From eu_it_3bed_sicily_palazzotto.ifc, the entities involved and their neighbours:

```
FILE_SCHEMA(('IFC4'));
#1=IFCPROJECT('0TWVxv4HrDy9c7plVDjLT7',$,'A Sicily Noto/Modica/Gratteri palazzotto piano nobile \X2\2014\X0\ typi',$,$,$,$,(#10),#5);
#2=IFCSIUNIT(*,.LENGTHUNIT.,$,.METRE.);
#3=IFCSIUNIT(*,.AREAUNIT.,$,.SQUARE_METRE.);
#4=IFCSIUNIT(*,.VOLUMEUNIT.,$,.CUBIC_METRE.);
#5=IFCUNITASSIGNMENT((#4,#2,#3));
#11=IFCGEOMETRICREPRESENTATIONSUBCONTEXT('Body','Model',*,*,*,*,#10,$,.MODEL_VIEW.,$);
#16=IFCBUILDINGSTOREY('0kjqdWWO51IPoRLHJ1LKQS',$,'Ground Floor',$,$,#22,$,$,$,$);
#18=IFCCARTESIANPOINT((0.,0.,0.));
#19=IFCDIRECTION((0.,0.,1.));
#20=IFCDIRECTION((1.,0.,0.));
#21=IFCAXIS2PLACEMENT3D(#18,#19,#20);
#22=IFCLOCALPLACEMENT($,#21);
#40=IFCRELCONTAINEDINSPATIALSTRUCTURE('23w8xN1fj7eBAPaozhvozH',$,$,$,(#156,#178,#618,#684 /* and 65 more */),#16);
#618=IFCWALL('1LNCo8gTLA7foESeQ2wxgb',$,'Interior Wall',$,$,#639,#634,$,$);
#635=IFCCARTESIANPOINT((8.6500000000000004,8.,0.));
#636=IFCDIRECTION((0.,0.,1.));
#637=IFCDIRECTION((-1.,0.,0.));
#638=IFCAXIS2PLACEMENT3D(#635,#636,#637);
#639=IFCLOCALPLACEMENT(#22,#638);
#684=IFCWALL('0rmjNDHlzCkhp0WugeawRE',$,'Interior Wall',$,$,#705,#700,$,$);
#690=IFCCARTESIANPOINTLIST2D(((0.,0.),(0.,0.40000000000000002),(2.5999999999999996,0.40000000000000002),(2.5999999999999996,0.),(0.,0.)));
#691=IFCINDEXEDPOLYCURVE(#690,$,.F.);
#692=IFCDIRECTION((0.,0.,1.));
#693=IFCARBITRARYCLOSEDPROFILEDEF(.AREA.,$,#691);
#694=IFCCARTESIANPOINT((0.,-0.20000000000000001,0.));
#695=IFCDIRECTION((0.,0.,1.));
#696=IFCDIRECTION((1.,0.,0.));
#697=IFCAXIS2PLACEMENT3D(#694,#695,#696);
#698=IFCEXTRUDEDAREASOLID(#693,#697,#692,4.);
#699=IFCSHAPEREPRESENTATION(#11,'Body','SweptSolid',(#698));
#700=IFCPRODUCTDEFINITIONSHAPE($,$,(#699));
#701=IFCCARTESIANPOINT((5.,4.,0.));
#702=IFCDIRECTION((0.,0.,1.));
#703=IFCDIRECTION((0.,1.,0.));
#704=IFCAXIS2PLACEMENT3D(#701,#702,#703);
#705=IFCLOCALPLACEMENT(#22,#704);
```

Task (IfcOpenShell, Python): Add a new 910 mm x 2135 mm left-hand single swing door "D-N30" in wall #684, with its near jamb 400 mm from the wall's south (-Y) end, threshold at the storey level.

```python
import numpy as np
import ifcopenshell
import ifcopenshell.api.feature
import ifcopenshell.api.geometry
import ifcopenshell.api.root
import ifcopenshell.api.spatial
import ifcopenshell.geom
import ifcopenshell.util.element
import ifcopenshell.util.placement
import ifcopenshell.util.representation
import ifcopenshell.util.shape
import ifcopenshell.util.unit

model = ifcopenshell.open("eu_it_3bed_sicily_palazzotto.ifc")
unit_scale = ifcopenshell.util.unit.calculate_unit_scale(model)
settings = ifcopenshell.geom.settings()


def volume(element):
    """Net volume in cubic metres, openings subtracted."""
    shape = ifcopenshell.geom.create_shape(settings, element)
    return ifcopenshell.util.shape.get_volume(shape.geometry)


wall = model.by_guid("0rmjNDHlzCkhp0WugeawRE")
storey = ifcopenshell.util.element.get_container(wall, ifc_class="IfcBuildingStorey")
context = ifcopenshell.util.representation.get_context(model, "Model", "Body", "MODEL_VIEW")
before = volume(wall)

width, height, from_end, sill = 0.91, 2.135, 0.4, 0.0  # metres

# The wall runs along its own X axis, and the end named is its -X end.
wall_shape = ifcopenshell.geom.create_shape(settings, wall)
x, y, z = ifcopenshell.util.shape.get_vertices(wall_shape.geometry).T
start = x.min() + from_end
face, thickness = float(y.min()), float(y.max() - y.min())
wall_matrix = ifcopenshell.util.placement.get_local_placement(wall.ObjectPlacement)
level = ifcopenshell.util.placement.get_local_placement(storey.ObjectPlacement)[2, 3]


def in_wall(x, y):
    """Placement at x, y metres in the wall's axes, at sill height."""
    matrix = wall_matrix.copy()
    matrix[:, 3] = wall_matrix @ np.array([x / unit_scale, y / unit_scale, 0.0, 1.0])
    matrix[2, 3] = level + sill / unit_scale
    return matrix


# Opening: a box that overshoots both wall faces by 50 mm.
opening = ifcopenshell.api.root.create_entity(model, ifc_class="IfcOpeningElement", predefined_type="OPENING")
box = ifcopenshell.api.geometry.add_wall_representation(
    model, context=context, length=width, height=height, thickness=thickness + 0.1
)
ifcopenshell.api.geometry.assign_representation(model, product=opening, representation=box)
ifcopenshell.api.geometry.edit_object_placement(model, product=opening, matrix=in_wall(start, face - 0.05), is_si=False)
ifcopenshell.api.feature.add_feature(model, feature=opening, element=wall)

door = ifcopenshell.api.root.create_entity(model, ifc_class="IfcDoor", name="D-N30", predefined_type="DOOR")
door.OverallWidth, door.OverallHeight = width / unit_scale, height / unit_scale
door.OperationType = "SINGLE_SWING_LEFT"
body = ifcopenshell.api.geometry.add_door_representation(
    model,
    context=context,
    overall_width=door.OverallWidth,
    overall_height=door.OverallHeight,
    operation_type="SINGLE_SWING_LEFT",
    lining_properties={"LiningDepth": thickness / unit_scale, "ThresholdDepth": thickness / unit_scale},
)
ifcopenshell.api.geometry.assign_representation(model, product=door, representation=body)
ifcopenshell.api.spatial.assign_container(model, products=[door], relating_structure=storey)
ifcopenshell.api.feature.add_filling(model, opening=opening, element=door)

# The lining spans the wall, so the door starts at the wall face.
ifcopenshell.api.geometry.edit_object_placement(model, product=door, matrix=in_wall(start, face), is_si=False)

after = volume(wall)

print(f"wall volume {before:.3f} -> {after:.3f} m3")

model.write("eu_it_3bed_sicily_palazzotto_edited.ifc")
```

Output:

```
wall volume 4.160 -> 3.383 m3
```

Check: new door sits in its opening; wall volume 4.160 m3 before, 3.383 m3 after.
